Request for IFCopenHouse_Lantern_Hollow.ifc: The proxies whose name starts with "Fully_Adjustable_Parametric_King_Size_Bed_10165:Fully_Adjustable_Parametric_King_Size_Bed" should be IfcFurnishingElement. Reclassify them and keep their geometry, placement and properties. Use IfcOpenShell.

First a look at what the model holds.

```python
import re

import ifcopenshell

model = ifcopenshell.open("IFCopenHouse_Lantern_Hollow.ifc")
print(model.schema)
seen = {}
for e in model.by_type("IfcBuildingElementProxy"):
    name = re.sub(r":\d+(:\d+)?$", "", e.Name or "")  # drop the element id that some exporters append
    seen[name] = seen.get(name, 0) + 1
for name, count in sorted(seen.items()):
    print(count, "x", name)
```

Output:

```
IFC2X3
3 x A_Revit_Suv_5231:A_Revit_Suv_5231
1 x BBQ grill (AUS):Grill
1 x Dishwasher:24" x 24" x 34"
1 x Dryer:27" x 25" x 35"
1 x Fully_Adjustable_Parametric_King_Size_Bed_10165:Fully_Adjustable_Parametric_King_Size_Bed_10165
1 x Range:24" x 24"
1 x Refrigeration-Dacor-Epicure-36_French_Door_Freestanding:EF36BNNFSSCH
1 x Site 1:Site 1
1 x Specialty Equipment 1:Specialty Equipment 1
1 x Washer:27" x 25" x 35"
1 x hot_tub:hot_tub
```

```python
import ifcopenshell
import ifcopenshell.api.root

model = ifcopenshell.open("IFCopenHouse_Lantern_Hollow.ifc")

proxies = [e.id() for e in model.by_type("IfcBuildingElementProxy") if (e.Name or "").startswith("Fully_Adjustable_Parametric_King_Size_Bed_10165:Fully_Adjustable_Parametric_King_Size_Bed")]
for step_id in proxies:
    proxy = model.by_id(step_id)
    ifcopenshell.api.root.reassign_class(model, product=proxy, ifc_class="IfcFurnishingElement")

print(sum(model.by_id(i).is_a("IfcFurnishingElement") for i in proxies), "reclassified")

model.write("IFCopenHouse_Lantern_Hollow_rev.ifc")
```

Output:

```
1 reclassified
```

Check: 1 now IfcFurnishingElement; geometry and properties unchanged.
